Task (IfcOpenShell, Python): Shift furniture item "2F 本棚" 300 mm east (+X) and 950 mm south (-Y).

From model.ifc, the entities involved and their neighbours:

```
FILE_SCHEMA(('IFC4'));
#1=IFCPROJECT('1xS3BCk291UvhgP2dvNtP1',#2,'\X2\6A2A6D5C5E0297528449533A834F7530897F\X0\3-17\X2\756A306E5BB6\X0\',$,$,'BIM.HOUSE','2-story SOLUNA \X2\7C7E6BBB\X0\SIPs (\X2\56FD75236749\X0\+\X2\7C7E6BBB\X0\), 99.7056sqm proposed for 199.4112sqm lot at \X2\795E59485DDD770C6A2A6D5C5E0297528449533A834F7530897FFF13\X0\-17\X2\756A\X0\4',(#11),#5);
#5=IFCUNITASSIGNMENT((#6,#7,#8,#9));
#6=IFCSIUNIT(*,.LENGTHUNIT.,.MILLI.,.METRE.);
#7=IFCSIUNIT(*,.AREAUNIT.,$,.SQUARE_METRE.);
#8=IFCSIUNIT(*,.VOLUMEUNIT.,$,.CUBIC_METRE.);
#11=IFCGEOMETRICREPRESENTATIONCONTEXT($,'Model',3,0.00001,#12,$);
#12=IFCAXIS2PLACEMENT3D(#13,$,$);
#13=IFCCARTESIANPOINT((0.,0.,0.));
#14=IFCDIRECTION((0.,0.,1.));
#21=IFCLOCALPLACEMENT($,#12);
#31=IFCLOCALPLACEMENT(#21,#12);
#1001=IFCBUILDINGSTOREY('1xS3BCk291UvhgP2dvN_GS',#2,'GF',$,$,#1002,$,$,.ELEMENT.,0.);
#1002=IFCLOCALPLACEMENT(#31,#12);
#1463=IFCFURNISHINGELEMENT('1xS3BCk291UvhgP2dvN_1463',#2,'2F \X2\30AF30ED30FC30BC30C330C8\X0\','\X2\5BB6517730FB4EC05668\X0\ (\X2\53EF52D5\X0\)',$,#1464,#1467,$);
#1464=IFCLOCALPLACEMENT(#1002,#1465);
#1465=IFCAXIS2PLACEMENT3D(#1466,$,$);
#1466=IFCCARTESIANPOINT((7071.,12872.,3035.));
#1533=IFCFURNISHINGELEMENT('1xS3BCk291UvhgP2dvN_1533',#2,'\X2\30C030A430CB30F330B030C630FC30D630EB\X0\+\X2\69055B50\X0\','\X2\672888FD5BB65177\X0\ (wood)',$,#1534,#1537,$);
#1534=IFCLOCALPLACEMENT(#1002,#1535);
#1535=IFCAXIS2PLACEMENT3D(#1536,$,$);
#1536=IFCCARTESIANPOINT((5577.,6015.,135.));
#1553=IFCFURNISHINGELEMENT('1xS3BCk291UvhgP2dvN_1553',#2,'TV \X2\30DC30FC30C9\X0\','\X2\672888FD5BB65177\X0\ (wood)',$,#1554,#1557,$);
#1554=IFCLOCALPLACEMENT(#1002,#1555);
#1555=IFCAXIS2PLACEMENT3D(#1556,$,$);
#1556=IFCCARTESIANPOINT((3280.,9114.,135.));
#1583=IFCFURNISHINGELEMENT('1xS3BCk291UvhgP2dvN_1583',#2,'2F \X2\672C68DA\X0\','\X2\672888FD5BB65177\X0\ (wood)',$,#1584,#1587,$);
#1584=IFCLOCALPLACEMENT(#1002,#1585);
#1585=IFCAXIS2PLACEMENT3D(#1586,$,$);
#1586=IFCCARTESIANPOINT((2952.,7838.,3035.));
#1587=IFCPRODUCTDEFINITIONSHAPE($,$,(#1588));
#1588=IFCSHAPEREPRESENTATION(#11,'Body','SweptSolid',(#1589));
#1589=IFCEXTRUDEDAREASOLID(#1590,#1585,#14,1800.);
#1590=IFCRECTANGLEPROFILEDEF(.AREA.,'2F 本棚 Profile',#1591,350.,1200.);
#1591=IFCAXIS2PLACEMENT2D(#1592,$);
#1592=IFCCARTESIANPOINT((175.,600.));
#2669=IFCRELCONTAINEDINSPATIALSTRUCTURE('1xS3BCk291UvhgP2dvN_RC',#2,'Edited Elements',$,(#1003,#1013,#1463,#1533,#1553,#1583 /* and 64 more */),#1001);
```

```python
import ifcopenshell
import ifcopenshell.api.geometry
import ifcopenshell.util.placement

model = ifcopenshell.open("model.ifc")

item = model.by_id(1583)
matrix = ifcopenshell.util.placement.get_local_placement(item.ObjectPlacement)
matrix[0, 3] += 300.0
matrix[1, 3] -= 950.0
ifcopenshell.api.geometry.edit_object_placement(model, product=item, matrix=matrix, is_si=False)

print(ifcopenshell.util.placement.get_local_placement(item.ObjectPlacement).round(3) + 0.0)

model.write("model_updated.ifc")
```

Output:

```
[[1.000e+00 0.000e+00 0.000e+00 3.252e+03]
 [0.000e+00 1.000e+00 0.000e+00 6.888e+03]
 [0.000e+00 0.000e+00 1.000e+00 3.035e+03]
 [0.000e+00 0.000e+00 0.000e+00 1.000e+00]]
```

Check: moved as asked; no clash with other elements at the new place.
